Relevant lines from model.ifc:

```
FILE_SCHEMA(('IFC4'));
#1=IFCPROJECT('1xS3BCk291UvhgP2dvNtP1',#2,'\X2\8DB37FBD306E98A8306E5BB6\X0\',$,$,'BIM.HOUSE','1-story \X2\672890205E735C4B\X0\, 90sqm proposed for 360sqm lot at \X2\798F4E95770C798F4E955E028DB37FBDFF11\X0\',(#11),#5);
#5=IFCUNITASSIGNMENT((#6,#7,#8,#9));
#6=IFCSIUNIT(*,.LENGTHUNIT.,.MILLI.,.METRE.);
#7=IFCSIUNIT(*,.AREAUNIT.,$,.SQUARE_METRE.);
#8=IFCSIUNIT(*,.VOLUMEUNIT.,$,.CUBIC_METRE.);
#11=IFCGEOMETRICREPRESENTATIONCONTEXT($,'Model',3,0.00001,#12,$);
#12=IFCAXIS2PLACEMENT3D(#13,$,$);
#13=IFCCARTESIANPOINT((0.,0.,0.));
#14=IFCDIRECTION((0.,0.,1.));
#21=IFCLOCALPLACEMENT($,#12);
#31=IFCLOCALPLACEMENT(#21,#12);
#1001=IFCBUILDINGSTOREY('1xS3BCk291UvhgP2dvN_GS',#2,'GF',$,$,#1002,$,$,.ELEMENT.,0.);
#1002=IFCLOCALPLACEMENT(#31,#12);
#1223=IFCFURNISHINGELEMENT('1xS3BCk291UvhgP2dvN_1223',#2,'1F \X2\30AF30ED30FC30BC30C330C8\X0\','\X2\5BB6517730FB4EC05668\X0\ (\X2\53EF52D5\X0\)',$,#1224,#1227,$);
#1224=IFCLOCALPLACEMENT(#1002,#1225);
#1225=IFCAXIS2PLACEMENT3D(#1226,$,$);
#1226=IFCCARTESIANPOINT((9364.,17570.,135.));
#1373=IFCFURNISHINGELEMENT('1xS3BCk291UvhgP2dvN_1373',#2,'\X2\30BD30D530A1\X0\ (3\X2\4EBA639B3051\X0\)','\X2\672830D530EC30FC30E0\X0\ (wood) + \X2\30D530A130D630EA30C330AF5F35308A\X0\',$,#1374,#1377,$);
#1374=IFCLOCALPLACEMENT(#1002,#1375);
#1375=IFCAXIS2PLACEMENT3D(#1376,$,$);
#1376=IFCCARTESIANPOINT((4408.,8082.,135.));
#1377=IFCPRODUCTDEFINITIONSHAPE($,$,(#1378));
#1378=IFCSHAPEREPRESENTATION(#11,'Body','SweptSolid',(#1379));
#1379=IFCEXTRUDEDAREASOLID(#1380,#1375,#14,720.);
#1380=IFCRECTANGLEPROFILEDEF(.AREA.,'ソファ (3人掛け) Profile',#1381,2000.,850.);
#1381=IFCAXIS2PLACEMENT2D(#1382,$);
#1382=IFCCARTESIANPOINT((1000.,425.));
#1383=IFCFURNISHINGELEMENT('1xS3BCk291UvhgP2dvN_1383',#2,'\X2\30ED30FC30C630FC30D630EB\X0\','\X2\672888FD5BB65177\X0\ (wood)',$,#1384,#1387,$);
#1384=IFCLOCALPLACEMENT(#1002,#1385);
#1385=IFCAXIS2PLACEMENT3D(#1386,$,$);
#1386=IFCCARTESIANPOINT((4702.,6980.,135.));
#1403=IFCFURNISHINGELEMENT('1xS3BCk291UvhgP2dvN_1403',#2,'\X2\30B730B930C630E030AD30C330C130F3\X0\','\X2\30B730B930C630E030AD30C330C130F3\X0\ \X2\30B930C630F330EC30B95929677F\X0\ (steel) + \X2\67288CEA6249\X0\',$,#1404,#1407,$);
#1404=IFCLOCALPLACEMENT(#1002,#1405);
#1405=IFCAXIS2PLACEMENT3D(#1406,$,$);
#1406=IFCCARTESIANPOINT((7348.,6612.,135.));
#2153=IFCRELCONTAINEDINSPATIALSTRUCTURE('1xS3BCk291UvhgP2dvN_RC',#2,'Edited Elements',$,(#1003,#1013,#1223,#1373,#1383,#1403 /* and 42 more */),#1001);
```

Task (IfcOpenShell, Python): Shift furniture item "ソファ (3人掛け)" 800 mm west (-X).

```python
import ifcopenshell
import ifcopenshell.api.geometry
import ifcopenshell.util.placement
import ifcopenshell.util.unit

model = ifcopenshell.open("model.ifc")
unit_scale = ifcopenshell.util.unit.calculate_unit_scale(model)

item = model.by_guid("1xS3BCk291UvhgP2dvN_1373")
matrix = ifcopenshell.util.placement.get_local_placement(item.ObjectPlacement)
matrix[0, 3] -= 0.8 / unit_scale
ifcopenshell.api.geometry.edit_object_placement(model, product=item, matrix=matrix, is_si=False)

print(ifcopenshell.util.placement.get_local_placement(item.ObjectPlacement).round(3) + 0.0)

model.write("model_updated.ifc")
```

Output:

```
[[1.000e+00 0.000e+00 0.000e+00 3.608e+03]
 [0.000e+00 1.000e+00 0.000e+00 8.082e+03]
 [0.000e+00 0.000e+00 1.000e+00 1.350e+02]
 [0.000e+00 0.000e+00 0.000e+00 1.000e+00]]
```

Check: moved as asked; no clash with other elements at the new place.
